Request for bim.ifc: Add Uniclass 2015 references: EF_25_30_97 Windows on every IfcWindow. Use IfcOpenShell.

First a look at what the model holds.

```python
import ifcopenshell

model = ifcopenshell.open("bim.ifc")
print(model.schema)
print("classifications:", [c.Name for c in model.by_type("IfcClassification")])
for ifc_class in ("IfcDoor", "IfcRoof", "IfcStair", "IfcWall", "IfcWindow"):
    print(ifc_class, len(model.by_type(ifc_class)))
```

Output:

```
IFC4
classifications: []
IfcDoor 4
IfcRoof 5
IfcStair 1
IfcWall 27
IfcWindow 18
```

```python
import ifcopenshell
import ifcopenshell.api.classification

model = ifcopenshell.open("bim.ifc")

system = ifcopenshell.api.classification.add_classification(model, classification="Uniclass 2015")

codes = {
    "IfcWindow": ("EF_25_30_97", "Windows"),
}
for ifc_class, (code, name) in codes.items():
    products = model.by_type(ifc_class)
    ifcopenshell.api.classification.add_reference(
        model, products=products, classification=system, identification=code, name=name
    )
    print(code, len(products))

model.write("bim_edited.ifc")
```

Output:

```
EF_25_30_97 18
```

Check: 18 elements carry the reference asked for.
